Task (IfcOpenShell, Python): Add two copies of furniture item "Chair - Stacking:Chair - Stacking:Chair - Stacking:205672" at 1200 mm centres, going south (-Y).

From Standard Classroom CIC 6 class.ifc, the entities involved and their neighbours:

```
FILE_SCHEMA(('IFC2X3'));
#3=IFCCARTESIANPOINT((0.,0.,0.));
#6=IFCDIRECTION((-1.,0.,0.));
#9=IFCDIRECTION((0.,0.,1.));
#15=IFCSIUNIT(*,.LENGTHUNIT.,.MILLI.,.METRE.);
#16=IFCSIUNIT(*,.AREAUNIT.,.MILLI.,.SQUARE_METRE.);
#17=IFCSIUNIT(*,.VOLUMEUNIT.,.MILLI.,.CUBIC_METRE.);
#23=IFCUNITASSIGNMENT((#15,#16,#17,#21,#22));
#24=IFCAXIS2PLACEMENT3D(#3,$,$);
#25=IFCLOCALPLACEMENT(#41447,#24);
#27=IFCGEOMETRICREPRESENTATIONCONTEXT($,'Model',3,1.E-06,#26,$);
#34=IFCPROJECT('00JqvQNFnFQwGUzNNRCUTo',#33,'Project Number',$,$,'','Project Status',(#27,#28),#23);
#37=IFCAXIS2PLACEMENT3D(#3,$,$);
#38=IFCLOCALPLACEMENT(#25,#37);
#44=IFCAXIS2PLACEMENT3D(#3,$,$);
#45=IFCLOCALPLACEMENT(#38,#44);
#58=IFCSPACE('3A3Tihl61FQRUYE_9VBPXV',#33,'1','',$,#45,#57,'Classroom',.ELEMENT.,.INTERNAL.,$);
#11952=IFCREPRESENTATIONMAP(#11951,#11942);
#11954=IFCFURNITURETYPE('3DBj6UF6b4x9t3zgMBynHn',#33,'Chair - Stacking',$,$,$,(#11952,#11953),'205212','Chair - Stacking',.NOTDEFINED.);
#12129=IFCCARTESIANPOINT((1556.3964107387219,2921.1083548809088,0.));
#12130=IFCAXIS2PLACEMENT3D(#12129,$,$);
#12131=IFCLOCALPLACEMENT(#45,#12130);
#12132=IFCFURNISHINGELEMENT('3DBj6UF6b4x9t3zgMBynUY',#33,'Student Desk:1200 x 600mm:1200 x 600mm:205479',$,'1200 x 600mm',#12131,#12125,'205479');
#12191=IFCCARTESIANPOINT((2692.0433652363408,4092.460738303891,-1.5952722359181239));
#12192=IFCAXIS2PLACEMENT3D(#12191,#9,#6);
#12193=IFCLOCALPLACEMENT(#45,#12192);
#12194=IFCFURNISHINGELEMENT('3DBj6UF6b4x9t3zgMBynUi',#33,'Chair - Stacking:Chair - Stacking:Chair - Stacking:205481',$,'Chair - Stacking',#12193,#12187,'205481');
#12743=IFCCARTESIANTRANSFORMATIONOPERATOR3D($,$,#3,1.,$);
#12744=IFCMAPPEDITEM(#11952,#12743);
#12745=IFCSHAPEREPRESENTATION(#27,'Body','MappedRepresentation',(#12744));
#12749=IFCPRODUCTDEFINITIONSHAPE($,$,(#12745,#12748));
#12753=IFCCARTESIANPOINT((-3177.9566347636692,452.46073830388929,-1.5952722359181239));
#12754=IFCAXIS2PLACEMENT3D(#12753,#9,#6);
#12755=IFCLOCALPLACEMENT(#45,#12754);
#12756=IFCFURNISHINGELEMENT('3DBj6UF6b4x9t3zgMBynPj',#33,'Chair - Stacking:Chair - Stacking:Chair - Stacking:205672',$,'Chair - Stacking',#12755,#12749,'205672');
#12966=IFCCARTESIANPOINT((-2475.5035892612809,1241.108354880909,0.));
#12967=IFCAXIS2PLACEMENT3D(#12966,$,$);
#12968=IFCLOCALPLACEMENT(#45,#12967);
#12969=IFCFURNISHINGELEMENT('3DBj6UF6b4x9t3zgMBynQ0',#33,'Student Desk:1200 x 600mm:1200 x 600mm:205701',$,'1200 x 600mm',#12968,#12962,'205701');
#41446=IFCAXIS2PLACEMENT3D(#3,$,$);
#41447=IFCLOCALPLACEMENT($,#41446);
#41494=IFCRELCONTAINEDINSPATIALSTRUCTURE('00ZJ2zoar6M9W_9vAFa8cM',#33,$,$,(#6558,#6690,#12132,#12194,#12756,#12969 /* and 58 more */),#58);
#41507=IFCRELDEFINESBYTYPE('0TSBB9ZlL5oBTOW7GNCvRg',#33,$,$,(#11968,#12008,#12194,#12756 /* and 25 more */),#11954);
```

```python
import numpy as np
import ifcopenshell
import ifcopenshell.api.geometry
import ifcopenshell.api.root
import ifcopenshell.util.element
import ifcopenshell.util.placement
import ifcopenshell.util.unit

model = ifcopenshell.open("Standard Classroom CIC 6 class.ifc")
unit_scale = ifcopenshell.util.unit.calculate_unit_scale(model)


def reuse_history(source, copy):
    """copy_class also copies each property set's owner history, people and application; keep the originals."""
    for rel in copy.IsDefinedBy:
        if rel.is_a("IfcRelDefinesByProperties") and (history := rel.RelatingPropertyDefinition.OwnerHistory):
            rel.RelatingPropertyDefinition.OwnerHistory = source.OwnerHistory
            ifcopenshell.util.element.remove_deep2(model, history)


source = model.by_guid("3DBj6UF6b4x9t3zgMBynPj")
base = ifcopenshell.util.placement.get_local_placement(source.ObjectPlacement)
step = np.array([0.0, -1.0, 0.0]) * 1.2 / unit_scale

for i in range(1, 3):
    copy = ifcopenshell.api.root.copy_class(model, product=source)
    copy.Representation = ifcopenshell.util.element.copy_deep(
        model, source.Representation, exclude=["IfcGeometricRepresentationContext", "IfcRepresentationMap"]
    )
    copy.Name = "Chair - Stacking:Chair - Stacking:Chair - Stacking"
    copy.Tag = None
    reuse_history(source, copy)
    matrix = base.copy()
    matrix[:3, 3] += i * step
    print("added at", matrix[:3, 3].round(3) + 0.0)
    ifcopenshell.api.geometry.edit_object_placement(model, product=copy, matrix=matrix, is_si=False)

model.write("Standard Classroom CIC 6 class_rev.ifc")
```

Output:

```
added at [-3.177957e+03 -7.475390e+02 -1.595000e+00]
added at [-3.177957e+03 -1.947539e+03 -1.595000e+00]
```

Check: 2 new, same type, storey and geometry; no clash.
